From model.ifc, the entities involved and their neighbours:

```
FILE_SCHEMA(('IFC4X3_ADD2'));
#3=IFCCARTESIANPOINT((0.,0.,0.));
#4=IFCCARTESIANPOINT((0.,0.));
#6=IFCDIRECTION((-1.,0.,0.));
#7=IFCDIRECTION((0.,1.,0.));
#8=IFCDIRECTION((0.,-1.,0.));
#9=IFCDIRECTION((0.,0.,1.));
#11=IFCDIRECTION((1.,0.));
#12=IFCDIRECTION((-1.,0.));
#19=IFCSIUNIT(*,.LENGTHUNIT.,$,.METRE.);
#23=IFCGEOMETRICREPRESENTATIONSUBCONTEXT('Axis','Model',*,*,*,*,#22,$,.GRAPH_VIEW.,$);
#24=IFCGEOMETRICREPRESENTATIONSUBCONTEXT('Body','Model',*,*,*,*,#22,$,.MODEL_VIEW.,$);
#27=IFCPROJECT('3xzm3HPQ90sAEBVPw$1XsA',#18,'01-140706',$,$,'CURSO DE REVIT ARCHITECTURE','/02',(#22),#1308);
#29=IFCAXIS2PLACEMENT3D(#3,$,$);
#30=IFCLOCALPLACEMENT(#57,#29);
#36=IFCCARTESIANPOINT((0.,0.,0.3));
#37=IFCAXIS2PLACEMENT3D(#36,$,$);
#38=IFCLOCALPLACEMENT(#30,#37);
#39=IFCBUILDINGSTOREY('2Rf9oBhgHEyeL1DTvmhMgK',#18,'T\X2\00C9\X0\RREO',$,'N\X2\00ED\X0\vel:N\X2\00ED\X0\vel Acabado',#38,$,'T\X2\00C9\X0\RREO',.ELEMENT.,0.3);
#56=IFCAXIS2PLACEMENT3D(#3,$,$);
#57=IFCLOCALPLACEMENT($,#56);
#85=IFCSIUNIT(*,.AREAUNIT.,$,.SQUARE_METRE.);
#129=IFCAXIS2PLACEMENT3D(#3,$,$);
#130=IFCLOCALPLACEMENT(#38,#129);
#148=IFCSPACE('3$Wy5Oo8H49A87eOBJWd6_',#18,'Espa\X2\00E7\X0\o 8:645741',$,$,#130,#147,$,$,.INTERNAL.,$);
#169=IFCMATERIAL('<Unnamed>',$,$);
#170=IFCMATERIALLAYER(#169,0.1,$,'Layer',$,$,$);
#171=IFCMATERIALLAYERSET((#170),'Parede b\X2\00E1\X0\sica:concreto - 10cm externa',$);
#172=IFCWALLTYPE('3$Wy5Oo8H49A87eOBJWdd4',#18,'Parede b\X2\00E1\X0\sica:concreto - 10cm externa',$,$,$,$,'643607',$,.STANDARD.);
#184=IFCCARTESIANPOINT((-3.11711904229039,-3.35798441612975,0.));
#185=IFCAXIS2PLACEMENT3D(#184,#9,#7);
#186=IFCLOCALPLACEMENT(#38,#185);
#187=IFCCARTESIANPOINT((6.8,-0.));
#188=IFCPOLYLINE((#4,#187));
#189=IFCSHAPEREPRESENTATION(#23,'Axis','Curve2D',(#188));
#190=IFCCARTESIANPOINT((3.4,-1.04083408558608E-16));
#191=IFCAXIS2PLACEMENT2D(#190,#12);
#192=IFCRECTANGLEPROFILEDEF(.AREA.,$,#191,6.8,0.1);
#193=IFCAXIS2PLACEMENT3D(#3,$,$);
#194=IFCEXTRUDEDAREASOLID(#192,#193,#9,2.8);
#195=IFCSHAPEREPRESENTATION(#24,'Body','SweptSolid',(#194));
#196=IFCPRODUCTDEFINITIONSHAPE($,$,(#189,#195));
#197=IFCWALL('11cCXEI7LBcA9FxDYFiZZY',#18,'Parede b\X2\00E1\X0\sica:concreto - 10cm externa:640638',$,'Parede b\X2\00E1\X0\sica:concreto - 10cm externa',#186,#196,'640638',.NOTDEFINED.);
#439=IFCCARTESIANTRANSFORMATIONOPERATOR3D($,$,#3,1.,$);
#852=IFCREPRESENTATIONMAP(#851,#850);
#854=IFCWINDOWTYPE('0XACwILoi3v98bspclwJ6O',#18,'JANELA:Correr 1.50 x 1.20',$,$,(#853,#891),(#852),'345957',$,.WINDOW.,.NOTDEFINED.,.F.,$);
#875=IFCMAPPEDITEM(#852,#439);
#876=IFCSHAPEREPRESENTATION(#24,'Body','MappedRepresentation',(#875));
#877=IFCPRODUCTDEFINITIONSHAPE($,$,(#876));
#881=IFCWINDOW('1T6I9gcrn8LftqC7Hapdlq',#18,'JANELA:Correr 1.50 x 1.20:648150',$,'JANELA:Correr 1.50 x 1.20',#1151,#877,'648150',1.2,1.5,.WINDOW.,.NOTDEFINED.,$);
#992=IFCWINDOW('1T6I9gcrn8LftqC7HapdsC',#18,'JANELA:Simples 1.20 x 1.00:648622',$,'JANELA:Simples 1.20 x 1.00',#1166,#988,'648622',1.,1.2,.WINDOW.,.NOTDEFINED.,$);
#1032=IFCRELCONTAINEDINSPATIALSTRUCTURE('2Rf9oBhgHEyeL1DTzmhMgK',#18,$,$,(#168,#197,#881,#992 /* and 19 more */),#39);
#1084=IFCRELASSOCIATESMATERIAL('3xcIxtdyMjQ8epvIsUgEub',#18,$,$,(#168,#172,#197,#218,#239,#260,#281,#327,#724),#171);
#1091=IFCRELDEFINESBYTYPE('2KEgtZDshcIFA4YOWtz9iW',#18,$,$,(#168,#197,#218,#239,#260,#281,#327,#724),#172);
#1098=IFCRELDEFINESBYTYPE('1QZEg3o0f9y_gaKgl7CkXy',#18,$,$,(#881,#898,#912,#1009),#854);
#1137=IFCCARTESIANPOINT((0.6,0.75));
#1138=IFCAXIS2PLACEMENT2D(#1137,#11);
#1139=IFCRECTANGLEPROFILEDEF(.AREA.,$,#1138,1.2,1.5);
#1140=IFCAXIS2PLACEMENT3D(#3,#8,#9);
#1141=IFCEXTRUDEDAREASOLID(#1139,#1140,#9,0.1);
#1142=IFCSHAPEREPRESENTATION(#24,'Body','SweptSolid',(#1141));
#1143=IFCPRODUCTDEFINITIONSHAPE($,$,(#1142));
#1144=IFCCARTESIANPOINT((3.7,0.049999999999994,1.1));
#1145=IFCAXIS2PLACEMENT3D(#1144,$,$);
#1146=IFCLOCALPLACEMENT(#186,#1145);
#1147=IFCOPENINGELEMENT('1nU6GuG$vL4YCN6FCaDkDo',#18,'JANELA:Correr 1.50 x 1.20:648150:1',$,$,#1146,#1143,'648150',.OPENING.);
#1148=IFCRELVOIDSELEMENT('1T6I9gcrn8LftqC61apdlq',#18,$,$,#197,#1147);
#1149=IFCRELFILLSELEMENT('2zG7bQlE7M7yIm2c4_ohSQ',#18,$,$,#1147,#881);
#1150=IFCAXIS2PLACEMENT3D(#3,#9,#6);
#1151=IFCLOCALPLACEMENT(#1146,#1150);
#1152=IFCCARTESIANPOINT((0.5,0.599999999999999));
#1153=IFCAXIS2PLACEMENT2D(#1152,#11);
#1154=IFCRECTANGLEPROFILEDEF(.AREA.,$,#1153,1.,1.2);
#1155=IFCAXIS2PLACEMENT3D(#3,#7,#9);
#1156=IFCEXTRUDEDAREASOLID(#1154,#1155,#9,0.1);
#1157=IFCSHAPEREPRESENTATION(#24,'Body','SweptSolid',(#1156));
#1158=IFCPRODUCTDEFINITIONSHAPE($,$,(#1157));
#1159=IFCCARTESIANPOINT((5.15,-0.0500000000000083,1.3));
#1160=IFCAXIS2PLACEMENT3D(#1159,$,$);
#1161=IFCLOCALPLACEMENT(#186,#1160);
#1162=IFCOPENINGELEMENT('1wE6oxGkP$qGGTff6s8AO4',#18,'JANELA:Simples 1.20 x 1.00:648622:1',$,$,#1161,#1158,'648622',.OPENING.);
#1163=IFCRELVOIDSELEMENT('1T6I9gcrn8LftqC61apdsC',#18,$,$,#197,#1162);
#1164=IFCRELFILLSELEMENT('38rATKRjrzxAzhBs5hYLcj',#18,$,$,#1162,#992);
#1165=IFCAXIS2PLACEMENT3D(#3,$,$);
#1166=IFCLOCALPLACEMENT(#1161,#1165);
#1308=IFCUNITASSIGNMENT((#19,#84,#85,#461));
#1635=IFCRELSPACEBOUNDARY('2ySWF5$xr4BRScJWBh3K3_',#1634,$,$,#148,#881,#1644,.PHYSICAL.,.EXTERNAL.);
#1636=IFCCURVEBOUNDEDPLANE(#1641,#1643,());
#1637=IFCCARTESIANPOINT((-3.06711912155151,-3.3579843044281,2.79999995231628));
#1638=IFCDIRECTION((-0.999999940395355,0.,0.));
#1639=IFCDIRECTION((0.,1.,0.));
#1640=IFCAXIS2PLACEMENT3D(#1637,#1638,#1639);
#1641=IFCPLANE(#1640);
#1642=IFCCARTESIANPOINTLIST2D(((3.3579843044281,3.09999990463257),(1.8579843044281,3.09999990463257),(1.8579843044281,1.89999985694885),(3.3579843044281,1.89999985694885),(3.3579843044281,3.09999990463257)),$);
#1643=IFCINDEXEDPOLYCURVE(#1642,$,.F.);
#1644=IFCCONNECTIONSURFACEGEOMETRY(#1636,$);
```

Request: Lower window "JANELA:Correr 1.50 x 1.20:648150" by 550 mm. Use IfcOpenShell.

```python
import numpy as np
import ifcopenshell
import ifcopenshell.api.geometry
import ifcopenshell.util.placement
import ifcopenshell.util.unit

model = ifcopenshell.open("model.ifc")
unit_scale = ifcopenshell.util.unit.calculate_unit_scale(model)

window = model.by_guid("1T6I9gcrn8LftqC7Hapdlq")
opening = window.FillsVoids[0].RelatingOpeningElement
dz = -0.55 / unit_scale

shift = np.array([0.0, 0.0, dz])
# The window is placed relative to its opening, so it follows when the opening moves.
matrix = ifcopenshell.util.placement.get_local_placement(opening.ObjectPlacement)
matrix[:3, 3] += shift
ifcopenshell.api.geometry.edit_object_placement(
    model, product=opening, matrix=matrix, is_si=False, should_transform_children=True
)

# Space boundary surfaces are stored in each space's coordinates; move them too.
for rel in window.ProvidesBoundaries:
    if not rel.ConnectionGeometry:
        continue
    surface = rel.ConnectionGeometry.SurfaceOnRelatingElement.BasisSurface
    space_matrix = ifcopenshell.util.placement.get_local_placement(rel.RelatingSpace.ObjectPlacement)
    point = np.array(surface.Position.Location.Coordinates) + space_matrix[:3, :3].T @ shift
    surface.Position = model.createIfcAxis2Placement3D(
        model.createIfcCartesianPoint(point.tolist()), surface.Position.Axis, surface.Position.RefDirection
    )

print(f"moved by {dz * unit_scale:+.3f} m")

model.write("model_edited.ifc")
```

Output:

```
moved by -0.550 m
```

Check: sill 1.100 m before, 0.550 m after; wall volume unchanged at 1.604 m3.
